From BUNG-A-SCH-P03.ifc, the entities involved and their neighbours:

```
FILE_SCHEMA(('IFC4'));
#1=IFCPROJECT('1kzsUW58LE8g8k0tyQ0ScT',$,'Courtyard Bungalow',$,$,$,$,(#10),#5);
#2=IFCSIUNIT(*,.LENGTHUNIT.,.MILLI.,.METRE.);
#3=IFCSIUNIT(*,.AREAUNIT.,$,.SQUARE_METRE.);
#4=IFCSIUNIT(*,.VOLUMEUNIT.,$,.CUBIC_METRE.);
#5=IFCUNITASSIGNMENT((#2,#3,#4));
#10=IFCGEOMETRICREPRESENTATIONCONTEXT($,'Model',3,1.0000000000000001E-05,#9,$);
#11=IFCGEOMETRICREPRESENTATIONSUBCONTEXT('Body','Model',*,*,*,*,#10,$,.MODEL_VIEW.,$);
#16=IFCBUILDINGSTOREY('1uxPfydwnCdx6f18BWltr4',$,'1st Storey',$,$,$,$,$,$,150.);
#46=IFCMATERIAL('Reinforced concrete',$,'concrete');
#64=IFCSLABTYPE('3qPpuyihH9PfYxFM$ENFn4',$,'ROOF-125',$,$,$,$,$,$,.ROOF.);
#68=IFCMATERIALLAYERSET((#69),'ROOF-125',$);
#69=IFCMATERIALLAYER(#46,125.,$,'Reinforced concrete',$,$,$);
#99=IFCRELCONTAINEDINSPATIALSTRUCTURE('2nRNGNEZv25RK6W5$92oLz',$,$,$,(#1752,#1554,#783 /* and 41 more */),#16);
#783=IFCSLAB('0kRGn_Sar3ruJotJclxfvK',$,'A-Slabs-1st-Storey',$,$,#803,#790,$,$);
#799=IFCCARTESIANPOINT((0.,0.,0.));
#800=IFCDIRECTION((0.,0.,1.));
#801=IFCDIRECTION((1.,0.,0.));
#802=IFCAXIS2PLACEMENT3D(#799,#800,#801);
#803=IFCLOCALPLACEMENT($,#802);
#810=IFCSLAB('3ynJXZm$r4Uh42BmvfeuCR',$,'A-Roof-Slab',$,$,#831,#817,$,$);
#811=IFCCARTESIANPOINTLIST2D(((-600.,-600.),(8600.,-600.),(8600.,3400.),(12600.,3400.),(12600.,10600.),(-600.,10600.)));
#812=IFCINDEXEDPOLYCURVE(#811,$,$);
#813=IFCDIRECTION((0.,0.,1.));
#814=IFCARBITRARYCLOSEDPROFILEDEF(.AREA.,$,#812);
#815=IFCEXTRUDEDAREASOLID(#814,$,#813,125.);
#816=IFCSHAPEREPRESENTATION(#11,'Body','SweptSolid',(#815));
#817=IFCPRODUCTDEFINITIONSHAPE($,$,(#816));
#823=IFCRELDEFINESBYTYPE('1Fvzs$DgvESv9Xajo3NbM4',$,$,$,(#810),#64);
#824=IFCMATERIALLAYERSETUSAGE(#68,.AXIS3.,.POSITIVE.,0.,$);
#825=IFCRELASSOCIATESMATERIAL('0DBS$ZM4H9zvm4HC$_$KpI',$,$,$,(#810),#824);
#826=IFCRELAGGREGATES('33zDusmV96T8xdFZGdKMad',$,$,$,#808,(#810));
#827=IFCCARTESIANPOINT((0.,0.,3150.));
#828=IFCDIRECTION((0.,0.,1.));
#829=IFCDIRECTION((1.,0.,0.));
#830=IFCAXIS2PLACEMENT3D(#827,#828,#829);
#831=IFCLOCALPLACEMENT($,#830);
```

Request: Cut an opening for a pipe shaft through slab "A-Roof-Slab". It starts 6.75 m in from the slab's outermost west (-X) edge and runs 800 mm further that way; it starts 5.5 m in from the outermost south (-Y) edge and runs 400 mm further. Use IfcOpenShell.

```python
import numpy as np
import ifcopenshell
import ifcopenshell.api.feature
import ifcopenshell.api.geometry
import ifcopenshell.api.root
import ifcopenshell.geom
import ifcopenshell.util.placement
import ifcopenshell.util.representation
import ifcopenshell.util.shape
import ifcopenshell.util.unit

model = ifcopenshell.open("BUNG-A-SCH-P03.ifc")
unit_scale = ifcopenshell.util.unit.calculate_unit_scale(model)
settings = ifcopenshell.geom.settings()


def volume(element):
    """Net volume in cubic metres, openings subtracted."""
    shape = ifcopenshell.geom.create_shape(settings, element)
    return ifcopenshell.util.shape.get_volume(shape.geometry)


slab = model.by_guid("3ynJXZm$r4Uh42BmvfeuCR")
before = volume(slab)

# Extent in the slab's own axes, in metres. The edges named are its -X and -Y sides.
slab_shape = ifcopenshell.geom.create_shape(settings, slab)
vertices = ifcopenshell.util.shape.get_vertices(slab_shape.geometry)
x_min, y_min, bottom = vertices.min(axis=0)
top = vertices[:, 2].max()

opening = ifcopenshell.api.root.create_entity(model, ifc_class="IfcOpeningElement", name="Pipe shaft opening", predefined_type="OPENING")
context = ifcopenshell.util.representation.get_context(model, "Model", "Body", "MODEL_VIEW")
width, depth = 0.8, 0.4
outline = [(0.0, 0.0), (width, 0.0), (width, depth), (0.0, depth), (0.0, 0.0)]
# Overshoot both faces by 50 mm so the cut is clean.
shape = ifcopenshell.api.geometry.add_slab_representation(
    model, context=context, depth=top - bottom + 0.1, polyline=outline
)
ifcopenshell.api.geometry.assign_representation(model, product=opening, representation=shape)

matrix = ifcopenshell.util.placement.get_local_placement(slab.ObjectPlacement)
matrix[:, 3] = matrix @ np.append(np.array([x_min + 6.75, y_min + 5.5, bottom - 0.05]) / unit_scale, 1.0)
ifcopenshell.api.geometry.edit_object_placement(model, product=opening, matrix=matrix, is_si=False)
ifcopenshell.api.feature.add_feature(model, feature=opening, element=slab)

after = volume(slab)

print(f"slab volume {before:.3f} -> {after:.3f} m3")

model.write("BUNG-A-SCH-P03-out.ifc")
```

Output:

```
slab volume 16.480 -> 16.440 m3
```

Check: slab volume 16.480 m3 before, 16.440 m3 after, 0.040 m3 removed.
